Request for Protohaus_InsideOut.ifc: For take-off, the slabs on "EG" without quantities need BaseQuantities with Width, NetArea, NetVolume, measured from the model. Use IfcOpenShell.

First a look at what the model holds.

```python
import ifcopenshell
import ifcopenshell.util.element
import ifcopenshell.util.unit

model = ifcopenshell.open("Protohaus_InsideOut.ifc")
print(model.schema)
for unit_type in ("LENGTHUNIT", "AREAUNIT", "VOLUMEUNIT"):
    print(unit_type, ifcopenshell.util.unit.calculate_unit_scale(model, unit_type))
storey = next(s for s in model.by_type("IfcBuildingStorey") if s.Name == "EG")
slabs = [e for e in ifcopenshell.util.element.get_decomposition(storey) if e.is_a("IfcSlab")]
for e in sorted(slabs, key=lambda e: e.id()):
    print(e.id(), e.is_a(), e.Name, list(ifcopenshell.util.element.get_psets(e, qtos_only=True)), sep=" | ")
```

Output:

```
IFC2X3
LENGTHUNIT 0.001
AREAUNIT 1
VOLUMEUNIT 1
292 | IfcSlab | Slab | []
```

```python
import ifcopenshell
import ifcopenshell.api.pset
import ifcopenshell.geom
import ifcopenshell.util.element
import ifcopenshell.util.shape
import ifcopenshell.util.unit

model = ifcopenshell.open("Protohaus_InsideOut.ifc")
unit_scale = ifcopenshell.util.unit.calculate_unit_scale(model)
area_scale = ifcopenshell.util.unit.calculate_unit_scale(model, "AREAUNIT")
volume_scale = ifcopenshell.util.unit.calculate_unit_scale(model, "VOLUMEUNIT")
settings = ifcopenshell.geom.settings()

storey = next(s for s in model.by_type("IfcBuildingStorey") if s.Name == "EG")
slabs = [e for e in ifcopenshell.util.element.get_decomposition(storey) if e.is_a("IfcSlab")]

for e in sorted(slabs, key=lambda e: e.id()):
    if ifcopenshell.util.element.get_psets(e, qtos_only=True, should_inherit=False):
        continue
    # Geometry comes back in metres, in the element's own axes.
    shape = ifcopenshell.geom.create_shape(settings, e)
    values = {
        "Width": ifcopenshell.util.shape.get_z(shape.geometry) / unit_scale,
        "NetArea": ifcopenshell.util.shape.get_footprint_area(shape.geometry) / area_scale,
        "NetVolume": ifcopenshell.util.shape.get_volume(shape.geometry) / volume_scale,
    }
    qto = ifcopenshell.api.pset.add_qto(model, product=e, name="BaseQuantities")
    ifcopenshell.api.pset.edit_qto(model, qto=qto, properties=values)
    print(e.id(), {k: round(v, 3) for k, v in values.items()})

model.write("Protohaus_InsideOut_v2.ifc")
```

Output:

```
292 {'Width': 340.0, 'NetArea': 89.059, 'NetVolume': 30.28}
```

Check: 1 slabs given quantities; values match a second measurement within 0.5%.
